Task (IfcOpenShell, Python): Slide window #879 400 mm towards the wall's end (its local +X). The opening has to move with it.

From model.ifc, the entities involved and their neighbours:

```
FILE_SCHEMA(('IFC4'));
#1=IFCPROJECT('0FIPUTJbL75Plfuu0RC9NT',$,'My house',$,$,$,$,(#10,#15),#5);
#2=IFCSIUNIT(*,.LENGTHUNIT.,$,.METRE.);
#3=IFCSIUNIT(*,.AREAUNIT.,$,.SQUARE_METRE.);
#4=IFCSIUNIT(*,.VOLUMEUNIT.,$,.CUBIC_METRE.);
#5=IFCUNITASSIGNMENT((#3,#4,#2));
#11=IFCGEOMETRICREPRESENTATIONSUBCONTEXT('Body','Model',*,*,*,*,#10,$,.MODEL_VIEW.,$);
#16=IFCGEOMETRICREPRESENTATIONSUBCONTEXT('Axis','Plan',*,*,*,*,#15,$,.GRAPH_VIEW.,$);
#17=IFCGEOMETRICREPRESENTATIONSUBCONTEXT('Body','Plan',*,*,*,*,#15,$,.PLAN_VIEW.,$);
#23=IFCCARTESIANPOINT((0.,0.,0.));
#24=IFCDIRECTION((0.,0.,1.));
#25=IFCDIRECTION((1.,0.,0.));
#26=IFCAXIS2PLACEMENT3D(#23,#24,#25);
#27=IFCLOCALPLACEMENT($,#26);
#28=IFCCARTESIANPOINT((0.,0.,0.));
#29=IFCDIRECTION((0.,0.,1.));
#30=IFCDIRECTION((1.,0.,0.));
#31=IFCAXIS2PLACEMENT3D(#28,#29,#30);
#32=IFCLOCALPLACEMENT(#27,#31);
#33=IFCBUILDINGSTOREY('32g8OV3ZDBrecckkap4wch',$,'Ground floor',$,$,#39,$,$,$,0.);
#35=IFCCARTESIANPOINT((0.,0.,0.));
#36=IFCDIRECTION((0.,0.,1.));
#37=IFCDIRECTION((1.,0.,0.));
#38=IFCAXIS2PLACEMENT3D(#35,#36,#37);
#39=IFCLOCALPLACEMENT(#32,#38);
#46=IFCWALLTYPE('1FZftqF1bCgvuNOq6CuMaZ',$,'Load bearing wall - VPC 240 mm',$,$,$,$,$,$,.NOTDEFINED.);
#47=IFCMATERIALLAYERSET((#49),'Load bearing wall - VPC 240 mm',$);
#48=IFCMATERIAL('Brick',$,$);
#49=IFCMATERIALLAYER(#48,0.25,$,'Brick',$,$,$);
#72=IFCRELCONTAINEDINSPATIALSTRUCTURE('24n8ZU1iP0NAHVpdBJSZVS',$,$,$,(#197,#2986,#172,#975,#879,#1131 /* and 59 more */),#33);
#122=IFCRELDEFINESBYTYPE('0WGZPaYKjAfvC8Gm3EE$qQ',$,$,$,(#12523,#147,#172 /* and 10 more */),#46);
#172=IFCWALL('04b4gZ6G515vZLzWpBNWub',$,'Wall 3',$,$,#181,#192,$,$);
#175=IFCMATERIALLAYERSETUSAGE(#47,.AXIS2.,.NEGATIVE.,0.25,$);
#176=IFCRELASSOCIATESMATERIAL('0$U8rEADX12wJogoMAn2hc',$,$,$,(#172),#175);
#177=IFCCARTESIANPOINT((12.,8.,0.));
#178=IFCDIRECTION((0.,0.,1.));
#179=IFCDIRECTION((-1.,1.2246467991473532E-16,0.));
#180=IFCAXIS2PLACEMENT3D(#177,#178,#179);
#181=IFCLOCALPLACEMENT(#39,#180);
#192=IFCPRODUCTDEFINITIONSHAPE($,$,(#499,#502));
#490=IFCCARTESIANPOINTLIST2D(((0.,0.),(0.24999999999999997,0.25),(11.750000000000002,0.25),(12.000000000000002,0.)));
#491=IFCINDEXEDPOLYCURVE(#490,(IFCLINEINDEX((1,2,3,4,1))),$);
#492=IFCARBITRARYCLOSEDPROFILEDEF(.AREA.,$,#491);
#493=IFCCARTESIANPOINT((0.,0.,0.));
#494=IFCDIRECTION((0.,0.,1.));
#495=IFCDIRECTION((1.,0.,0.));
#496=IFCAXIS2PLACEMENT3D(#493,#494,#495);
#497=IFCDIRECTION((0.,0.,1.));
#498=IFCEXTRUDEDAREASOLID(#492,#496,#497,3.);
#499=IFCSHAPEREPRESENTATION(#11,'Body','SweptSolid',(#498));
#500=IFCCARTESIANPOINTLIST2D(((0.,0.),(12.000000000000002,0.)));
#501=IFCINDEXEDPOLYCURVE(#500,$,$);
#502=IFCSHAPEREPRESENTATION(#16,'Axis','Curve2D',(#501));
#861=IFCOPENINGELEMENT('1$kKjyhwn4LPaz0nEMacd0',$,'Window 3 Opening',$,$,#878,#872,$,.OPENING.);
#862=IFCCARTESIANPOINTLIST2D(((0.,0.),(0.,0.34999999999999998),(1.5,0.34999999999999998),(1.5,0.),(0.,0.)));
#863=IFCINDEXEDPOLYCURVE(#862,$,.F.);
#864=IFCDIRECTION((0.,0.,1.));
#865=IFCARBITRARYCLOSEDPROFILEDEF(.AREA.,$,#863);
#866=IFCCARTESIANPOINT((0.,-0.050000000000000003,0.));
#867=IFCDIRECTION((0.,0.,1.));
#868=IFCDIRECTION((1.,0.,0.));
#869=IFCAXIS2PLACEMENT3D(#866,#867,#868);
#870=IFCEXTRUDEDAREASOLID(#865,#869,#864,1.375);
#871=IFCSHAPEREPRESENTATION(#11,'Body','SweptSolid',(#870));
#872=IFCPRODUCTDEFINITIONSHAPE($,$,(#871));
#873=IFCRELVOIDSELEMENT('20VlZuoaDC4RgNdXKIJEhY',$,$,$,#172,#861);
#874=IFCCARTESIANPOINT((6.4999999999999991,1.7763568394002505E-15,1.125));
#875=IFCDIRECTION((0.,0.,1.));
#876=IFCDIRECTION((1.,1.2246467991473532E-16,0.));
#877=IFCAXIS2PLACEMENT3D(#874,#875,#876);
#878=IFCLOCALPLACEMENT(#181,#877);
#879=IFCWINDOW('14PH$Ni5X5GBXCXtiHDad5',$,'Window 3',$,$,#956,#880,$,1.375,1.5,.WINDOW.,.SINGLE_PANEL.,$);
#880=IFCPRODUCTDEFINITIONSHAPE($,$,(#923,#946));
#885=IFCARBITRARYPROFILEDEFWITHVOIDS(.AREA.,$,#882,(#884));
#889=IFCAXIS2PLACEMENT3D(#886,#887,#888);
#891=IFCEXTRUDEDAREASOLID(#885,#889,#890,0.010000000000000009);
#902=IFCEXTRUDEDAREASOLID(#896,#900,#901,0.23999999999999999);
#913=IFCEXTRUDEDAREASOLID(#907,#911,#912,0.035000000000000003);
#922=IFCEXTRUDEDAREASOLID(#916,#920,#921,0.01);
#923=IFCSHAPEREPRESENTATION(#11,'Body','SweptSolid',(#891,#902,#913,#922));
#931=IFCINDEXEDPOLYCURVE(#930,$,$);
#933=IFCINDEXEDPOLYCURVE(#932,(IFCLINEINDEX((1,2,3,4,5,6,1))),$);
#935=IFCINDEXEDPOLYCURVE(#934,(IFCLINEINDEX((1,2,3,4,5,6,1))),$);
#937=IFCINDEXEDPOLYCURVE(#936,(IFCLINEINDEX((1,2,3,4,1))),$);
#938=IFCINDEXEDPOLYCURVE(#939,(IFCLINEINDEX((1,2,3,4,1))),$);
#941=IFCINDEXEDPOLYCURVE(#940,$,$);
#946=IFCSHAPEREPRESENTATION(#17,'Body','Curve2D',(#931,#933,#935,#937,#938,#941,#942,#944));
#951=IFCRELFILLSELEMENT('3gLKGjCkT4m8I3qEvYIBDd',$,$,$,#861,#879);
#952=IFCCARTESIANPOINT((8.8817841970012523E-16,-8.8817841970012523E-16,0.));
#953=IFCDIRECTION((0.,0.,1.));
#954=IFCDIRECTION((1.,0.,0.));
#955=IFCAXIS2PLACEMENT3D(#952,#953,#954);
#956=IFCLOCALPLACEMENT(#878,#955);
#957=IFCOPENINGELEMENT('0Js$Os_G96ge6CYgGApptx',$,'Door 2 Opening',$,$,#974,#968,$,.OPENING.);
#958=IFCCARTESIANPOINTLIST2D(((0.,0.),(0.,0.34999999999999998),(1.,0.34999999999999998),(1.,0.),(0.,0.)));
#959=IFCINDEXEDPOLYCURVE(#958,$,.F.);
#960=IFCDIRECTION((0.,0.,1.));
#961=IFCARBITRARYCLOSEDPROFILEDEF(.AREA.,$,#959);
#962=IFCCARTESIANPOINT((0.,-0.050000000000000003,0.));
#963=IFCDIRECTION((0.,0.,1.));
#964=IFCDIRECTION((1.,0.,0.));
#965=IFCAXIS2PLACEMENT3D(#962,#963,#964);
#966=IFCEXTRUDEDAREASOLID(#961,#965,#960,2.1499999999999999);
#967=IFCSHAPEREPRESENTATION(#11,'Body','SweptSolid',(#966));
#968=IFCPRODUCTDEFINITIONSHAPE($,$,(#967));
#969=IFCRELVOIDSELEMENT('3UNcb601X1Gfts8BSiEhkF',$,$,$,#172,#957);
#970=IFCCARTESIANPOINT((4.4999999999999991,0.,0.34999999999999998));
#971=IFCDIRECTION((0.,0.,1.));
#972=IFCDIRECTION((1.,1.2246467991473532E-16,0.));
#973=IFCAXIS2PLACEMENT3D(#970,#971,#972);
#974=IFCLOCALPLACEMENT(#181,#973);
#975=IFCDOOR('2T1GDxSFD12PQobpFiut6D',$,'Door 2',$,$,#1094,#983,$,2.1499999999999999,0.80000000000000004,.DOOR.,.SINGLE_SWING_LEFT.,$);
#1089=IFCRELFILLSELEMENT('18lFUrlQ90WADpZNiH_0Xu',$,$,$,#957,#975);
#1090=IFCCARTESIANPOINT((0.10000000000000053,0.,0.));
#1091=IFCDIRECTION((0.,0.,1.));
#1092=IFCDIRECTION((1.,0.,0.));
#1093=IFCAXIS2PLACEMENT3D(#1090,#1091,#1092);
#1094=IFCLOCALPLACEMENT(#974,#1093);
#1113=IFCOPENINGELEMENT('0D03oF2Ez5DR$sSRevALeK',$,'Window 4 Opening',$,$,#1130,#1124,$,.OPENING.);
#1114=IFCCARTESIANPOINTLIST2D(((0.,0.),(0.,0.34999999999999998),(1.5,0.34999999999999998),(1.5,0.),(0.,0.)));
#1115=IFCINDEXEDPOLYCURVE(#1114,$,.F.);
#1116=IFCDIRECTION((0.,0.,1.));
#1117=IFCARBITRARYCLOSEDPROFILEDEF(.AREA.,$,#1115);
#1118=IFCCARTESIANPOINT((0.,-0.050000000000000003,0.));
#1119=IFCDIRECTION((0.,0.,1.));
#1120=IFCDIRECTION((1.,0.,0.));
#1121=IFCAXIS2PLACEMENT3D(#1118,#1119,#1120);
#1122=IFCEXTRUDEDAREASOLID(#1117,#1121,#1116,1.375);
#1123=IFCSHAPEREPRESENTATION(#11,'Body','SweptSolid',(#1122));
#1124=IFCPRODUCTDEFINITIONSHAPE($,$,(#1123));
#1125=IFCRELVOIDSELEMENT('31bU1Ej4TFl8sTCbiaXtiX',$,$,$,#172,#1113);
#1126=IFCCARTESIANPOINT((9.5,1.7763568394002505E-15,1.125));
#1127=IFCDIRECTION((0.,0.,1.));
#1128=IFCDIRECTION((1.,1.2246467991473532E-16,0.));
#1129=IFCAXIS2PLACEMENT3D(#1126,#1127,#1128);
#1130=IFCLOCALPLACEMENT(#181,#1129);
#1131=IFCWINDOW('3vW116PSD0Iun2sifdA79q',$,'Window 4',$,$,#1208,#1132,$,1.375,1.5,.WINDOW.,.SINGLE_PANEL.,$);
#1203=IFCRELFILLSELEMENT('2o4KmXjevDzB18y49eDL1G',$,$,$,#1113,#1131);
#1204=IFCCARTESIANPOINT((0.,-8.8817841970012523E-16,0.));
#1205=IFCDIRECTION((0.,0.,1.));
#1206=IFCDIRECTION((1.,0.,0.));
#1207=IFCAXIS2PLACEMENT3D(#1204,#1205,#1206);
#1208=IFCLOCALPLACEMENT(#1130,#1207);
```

```python
import ifcopenshell
import ifcopenshell.api.geometry
import ifcopenshell.util.placement

model = ifcopenshell.open("model.ifc")

window = model.by_guid("14PH$Ni5X5GBXCXtiHDad5")
opening = window.FillsVoids[0].RelatingOpeningElement
wall = opening.VoidsElements[0].RelatingBuildingElement

wall_matrix = ifcopenshell.util.placement.get_local_placement(wall.ObjectPlacement)
shift = wall_matrix[:3, 0] * 0.4
before = ifcopenshell.util.placement.get_local_placement(window.ObjectPlacement)[:3, 3].copy()

# The window is placed relative to its opening, so it follows when the opening moves.
matrix = ifcopenshell.util.placement.get_local_placement(opening.ObjectPlacement)
matrix[:3, 3] += shift
ifcopenshell.api.geometry.edit_object_placement(
    model, product=opening, matrix=matrix, is_si=False, should_transform_children=True
)

after = ifcopenshell.util.placement.get_local_placement(window.ObjectPlacement)[:3, 3]
print("window moved by", (after - before).round(3) + 0.0)

model.write("model_rev.ifc")
```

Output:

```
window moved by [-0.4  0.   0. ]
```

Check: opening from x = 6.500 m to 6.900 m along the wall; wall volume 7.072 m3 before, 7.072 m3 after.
